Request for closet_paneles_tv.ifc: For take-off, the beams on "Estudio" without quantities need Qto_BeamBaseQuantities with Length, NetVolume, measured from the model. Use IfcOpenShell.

First a look at what the model holds.

```python
import ifcopenshell
import ifcopenshell.util.element
import ifcopenshell.util.unit

model = ifcopenshell.open("closet_paneles_tv.ifc")
print(model.schema)
for unit_type in ("LENGTHUNIT", "AREAUNIT", "VOLUMEUNIT"):
    print(unit_type, ifcopenshell.util.unit.calculate_unit_scale(model, unit_type))
storey = next(s for s in model.by_type("IfcBuildingStorey") if s.Name == "Estudio")
beams = [e for e in ifcopenshell.util.element.get_decomposition(storey) if e.is_a("IfcBeam")]
for e in sorted(beams, key=lambda e: e.id()):
    print(e.id(), e.is_a(), e.Name, list(ifcopenshell.util.element.get_psets(e, qtos_only=True)), sep=" | ")
```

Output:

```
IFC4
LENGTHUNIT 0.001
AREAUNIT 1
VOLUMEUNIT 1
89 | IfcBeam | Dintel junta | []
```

```python
import ifcopenshell
import ifcopenshell.api.pset
import ifcopenshell.geom
import ifcopenshell.util.element
import ifcopenshell.util.shape
import ifcopenshell.util.unit

model = ifcopenshell.open("closet_paneles_tv.ifc")
unit_scale = ifcopenshell.util.unit.calculate_unit_scale(model)
volume_scale = ifcopenshell.util.unit.calculate_unit_scale(model, "VOLUMEUNIT")
settings = ifcopenshell.geom.settings()

storey = next(s for s in model.by_type("IfcBuildingStorey") if s.Name == "Estudio")
beams = [e for e in ifcopenshell.util.element.get_decomposition(storey) if e.is_a("IfcBeam")]

for e in sorted(beams, key=lambda e: e.id()):
    if ifcopenshell.util.element.get_psets(e, qtos_only=True, should_inherit=False):
        continue
    # Geometry comes back in metres, in the element's own axes.
    shape = ifcopenshell.geom.create_shape(settings, e)
    values = {
        "Length": ifcopenshell.util.shape.get_max_xyz(shape.geometry) / unit_scale,
        "NetVolume": ifcopenshell.util.shape.get_volume(shape.geometry) / volume_scale,
    }
    qto = ifcopenshell.api.pset.add_qto(model, product=e, name="Qto_BeamBaseQuantities")
    ifcopenshell.api.pset.edit_qto(model, qto=qto, properties=values)
    print(e.id(), {k: round(v, 3) for k, v in values.items()})

model.write("closet_paneles_tv_updated.ifc")
```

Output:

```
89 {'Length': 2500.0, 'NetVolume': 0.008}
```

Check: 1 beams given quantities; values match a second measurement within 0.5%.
